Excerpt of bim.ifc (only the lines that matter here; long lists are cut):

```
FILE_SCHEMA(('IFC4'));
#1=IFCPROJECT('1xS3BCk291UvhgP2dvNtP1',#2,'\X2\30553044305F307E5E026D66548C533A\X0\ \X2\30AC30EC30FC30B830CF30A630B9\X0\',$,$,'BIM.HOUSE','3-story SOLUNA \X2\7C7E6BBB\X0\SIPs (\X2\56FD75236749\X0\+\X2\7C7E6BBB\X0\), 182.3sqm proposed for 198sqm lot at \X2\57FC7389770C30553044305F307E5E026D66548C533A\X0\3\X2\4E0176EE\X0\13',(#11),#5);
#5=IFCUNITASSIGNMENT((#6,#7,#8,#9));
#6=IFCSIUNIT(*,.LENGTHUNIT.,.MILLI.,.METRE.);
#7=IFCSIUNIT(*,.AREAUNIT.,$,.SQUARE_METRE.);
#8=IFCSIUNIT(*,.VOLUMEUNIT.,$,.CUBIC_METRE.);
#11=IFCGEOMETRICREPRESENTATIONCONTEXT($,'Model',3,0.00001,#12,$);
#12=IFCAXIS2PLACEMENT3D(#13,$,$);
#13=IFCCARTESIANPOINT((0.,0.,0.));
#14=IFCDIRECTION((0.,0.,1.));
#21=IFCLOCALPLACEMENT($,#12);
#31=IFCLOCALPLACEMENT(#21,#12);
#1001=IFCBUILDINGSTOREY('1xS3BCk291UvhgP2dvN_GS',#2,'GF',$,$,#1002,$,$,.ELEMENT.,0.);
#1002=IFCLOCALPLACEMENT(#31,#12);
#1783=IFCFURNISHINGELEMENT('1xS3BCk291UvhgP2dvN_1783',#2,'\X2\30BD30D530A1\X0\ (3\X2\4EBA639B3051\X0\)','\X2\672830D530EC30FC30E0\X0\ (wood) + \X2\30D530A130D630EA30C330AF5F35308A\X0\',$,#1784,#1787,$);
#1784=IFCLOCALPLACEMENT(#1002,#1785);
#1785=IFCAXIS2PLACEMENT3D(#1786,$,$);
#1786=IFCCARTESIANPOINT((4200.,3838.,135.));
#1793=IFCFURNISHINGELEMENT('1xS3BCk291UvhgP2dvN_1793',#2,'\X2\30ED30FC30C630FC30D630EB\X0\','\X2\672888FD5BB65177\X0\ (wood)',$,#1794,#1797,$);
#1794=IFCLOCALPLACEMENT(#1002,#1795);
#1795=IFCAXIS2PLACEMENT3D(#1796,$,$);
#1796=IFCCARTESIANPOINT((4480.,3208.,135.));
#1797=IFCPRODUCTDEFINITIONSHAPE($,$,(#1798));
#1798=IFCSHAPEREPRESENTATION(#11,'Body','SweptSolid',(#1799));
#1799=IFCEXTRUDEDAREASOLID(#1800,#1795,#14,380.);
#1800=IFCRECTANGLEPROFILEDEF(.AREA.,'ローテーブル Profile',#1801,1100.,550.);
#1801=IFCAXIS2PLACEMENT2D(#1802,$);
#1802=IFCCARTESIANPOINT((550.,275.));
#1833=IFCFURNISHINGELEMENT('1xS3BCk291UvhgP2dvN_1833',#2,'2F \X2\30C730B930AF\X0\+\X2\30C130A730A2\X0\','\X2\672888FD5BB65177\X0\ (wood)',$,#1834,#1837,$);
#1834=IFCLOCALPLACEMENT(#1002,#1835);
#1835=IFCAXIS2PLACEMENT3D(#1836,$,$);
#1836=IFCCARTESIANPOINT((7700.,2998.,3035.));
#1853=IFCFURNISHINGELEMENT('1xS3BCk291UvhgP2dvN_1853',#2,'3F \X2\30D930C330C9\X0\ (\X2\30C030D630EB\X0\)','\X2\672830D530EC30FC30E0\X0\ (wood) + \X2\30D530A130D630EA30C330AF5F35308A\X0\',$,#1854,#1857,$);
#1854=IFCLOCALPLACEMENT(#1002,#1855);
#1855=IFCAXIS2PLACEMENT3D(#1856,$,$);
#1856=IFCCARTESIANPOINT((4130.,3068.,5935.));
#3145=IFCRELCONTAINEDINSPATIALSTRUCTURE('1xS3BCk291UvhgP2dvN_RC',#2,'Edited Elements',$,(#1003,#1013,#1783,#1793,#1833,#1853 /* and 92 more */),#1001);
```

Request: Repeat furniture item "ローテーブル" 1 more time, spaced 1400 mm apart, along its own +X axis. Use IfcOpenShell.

```python
import ifcopenshell
import ifcopenshell.api.geometry
import ifcopenshell.api.root
import ifcopenshell.util.element
import ifcopenshell.util.placement

model = ifcopenshell.open("bim.ifc")


def reuse_history(source, copy):
    """copy_class also copies each property set's owner history, people and application; keep the originals."""
    for rel in copy.IsDefinedBy:
        if rel.is_a("IfcRelDefinesByProperties") and (history := rel.RelatingPropertyDefinition.OwnerHistory):
            rel.RelatingPropertyDefinition.OwnerHistory = source.OwnerHistory
            ifcopenshell.util.element.remove_deep2(model, history)


source = model.by_guid("1xS3BCk291UvhgP2dvN_1793")
base = ifcopenshell.util.placement.get_local_placement(source.ObjectPlacement)
step = base[:3, 0] * 1400.0

for i in range(1, 2):
    copy = ifcopenshell.api.root.copy_class(model, product=source)
    copy.Representation = ifcopenshell.util.element.copy_deep(
        model, source.Representation, exclude=["IfcGeometricRepresentationContext", "IfcRepresentationMap"]
    )
    reuse_history(source, copy)
    matrix = base.copy()
    matrix[:3, 3] += i * step
    print("added at", matrix[:3, 3].round(3) + 0.0)
    ifcopenshell.api.geometry.edit_object_placement(model, product=copy, matrix=matrix, is_si=False)

model.write("bim_updated.ifc")
```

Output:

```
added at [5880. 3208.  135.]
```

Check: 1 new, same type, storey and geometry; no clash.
